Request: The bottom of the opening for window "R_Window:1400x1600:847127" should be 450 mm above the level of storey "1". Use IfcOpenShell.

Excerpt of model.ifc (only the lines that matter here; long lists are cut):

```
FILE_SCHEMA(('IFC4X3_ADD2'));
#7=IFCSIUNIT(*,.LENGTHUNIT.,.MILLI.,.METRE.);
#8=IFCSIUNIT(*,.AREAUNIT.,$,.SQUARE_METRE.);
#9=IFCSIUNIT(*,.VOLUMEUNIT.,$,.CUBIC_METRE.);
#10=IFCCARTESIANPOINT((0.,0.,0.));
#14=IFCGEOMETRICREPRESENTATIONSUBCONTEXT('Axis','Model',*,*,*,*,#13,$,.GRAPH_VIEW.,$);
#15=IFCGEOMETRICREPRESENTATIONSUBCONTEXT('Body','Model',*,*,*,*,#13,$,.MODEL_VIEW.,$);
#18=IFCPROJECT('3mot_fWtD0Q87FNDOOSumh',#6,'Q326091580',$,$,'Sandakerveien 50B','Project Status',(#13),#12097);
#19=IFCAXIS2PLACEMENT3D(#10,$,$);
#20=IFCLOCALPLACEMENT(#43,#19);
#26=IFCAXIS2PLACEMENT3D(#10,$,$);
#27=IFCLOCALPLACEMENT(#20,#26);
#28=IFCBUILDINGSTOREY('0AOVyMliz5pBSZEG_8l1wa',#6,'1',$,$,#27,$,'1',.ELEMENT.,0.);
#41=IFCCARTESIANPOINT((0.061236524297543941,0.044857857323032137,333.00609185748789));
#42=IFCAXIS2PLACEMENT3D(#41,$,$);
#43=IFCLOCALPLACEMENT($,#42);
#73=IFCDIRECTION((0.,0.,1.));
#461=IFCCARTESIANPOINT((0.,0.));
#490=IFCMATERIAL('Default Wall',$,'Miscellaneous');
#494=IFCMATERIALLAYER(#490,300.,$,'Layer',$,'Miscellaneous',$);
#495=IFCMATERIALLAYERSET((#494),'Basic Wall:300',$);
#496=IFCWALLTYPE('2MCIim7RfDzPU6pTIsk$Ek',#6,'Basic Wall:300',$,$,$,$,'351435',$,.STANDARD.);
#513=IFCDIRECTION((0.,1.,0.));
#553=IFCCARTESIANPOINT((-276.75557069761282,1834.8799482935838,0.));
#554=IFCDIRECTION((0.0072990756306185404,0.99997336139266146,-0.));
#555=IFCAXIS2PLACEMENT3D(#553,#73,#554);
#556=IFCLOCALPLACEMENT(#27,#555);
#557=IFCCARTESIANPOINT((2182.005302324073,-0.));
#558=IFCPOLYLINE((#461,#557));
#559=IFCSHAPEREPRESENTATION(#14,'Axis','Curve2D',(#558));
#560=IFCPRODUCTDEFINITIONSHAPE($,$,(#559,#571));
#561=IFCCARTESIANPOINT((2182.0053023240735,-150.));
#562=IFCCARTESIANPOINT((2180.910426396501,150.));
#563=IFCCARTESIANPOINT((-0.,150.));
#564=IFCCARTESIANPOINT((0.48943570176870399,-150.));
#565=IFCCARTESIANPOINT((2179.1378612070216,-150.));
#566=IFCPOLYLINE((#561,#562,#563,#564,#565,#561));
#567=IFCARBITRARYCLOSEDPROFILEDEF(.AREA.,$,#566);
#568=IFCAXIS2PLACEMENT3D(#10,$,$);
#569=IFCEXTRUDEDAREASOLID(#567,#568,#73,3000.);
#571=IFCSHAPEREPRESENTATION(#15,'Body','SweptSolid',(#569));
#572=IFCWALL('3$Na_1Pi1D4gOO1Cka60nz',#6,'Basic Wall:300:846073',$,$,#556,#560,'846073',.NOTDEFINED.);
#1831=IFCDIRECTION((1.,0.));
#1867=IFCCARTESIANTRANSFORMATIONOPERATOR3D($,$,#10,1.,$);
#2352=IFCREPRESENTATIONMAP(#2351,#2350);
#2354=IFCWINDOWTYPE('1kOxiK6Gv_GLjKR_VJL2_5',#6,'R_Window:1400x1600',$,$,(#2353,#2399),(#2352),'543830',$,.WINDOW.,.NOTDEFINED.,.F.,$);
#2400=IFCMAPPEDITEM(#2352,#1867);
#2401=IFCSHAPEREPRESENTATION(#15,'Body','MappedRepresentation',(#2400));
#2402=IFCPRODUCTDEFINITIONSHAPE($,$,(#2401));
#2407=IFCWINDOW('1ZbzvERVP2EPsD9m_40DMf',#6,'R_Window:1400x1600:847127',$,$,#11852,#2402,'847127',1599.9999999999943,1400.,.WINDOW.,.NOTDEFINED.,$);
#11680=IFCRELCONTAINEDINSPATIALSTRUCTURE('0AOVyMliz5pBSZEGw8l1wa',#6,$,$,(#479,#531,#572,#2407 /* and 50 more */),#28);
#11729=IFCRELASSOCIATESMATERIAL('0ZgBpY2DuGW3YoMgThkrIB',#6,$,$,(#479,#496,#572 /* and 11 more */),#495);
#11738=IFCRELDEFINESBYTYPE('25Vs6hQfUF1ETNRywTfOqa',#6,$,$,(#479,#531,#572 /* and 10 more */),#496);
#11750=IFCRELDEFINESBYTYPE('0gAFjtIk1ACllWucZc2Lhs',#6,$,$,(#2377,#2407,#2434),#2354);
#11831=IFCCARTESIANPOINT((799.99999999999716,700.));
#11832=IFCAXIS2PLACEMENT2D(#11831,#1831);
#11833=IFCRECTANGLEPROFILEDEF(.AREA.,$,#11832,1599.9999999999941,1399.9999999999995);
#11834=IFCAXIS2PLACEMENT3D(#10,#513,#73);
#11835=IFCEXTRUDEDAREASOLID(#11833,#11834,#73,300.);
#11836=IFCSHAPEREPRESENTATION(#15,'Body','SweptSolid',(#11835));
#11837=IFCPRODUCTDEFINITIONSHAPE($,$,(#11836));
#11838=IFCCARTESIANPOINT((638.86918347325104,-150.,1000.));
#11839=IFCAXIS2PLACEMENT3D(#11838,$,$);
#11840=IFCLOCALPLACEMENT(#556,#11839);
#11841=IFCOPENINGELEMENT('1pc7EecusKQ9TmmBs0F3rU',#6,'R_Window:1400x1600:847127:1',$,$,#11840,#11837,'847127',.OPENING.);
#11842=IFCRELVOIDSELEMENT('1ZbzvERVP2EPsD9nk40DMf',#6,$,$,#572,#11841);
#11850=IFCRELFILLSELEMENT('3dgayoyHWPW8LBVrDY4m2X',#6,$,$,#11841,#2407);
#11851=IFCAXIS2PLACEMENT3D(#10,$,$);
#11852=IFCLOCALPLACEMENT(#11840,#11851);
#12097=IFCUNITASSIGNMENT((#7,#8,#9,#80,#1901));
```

```python
import numpy as np
import ifcopenshell
import ifcopenshell.api.geometry
import ifcopenshell.geom
import ifcopenshell.util.element
import ifcopenshell.util.placement
import ifcopenshell.util.shape
import ifcopenshell.util.unit

model = ifcopenshell.open("model.ifc")
unit_scale = ifcopenshell.util.unit.calculate_unit_scale(model)

window = model.by_guid("1ZbzvERVP2EPsD9m_40DMf")
opening = window.FillsVoids[0].RelatingOpeningElement
storey = ifcopenshell.util.element.get_container(window, ifc_class="IfcBuildingStorey")
level = ifcopenshell.util.placement.get_local_placement(storey.ObjectPlacement)[2, 3]

# The opening's origin need not be at the sill, so measure its lowest point.
shape = ifcopenshell.geom.create_shape(ifcopenshell.geom.settings(), opening)
bottom = ifcopenshell.util.shape.get_shape_bottom_elevation(shape, shape.geometry) / unit_scale
dz = level + 0.45 / unit_scale - bottom

shift = np.array([0.0, 0.0, dz])
# The window is placed relative to its opening, so it follows when the opening moves.
matrix = ifcopenshell.util.placement.get_local_placement(opening.ObjectPlacement)
matrix[:3, 3] += shift
ifcopenshell.api.geometry.edit_object_placement(
    model, product=opening, matrix=matrix, is_si=False, should_transform_children=True
)

print(f"moved by {dz * unit_scale:+.3f} m")

model.write("model_v2.ifc")
```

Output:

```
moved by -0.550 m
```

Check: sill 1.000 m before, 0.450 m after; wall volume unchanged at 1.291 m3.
